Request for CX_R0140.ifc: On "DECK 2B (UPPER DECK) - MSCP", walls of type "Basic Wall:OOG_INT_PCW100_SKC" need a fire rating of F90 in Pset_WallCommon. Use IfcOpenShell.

First a look at what the model holds.

```python
import ifcopenshell
import ifcopenshell.util.element

model = ifcopenshell.open("CX_R0140.ifc")
print(model.schema)
storey = next(s for s in model.by_type("IfcBuildingStorey") if s.Name == "DECK 2B (UPPER DECK) - MSCP")
walls = [e for e in ifcopenshell.util.element.get_decomposition(storey) if e.is_a("IfcWall")]
seen = {}
for e in walls:
    element_type = ifcopenshell.util.element.get_type(e)
    key = (element_type.Name if element_type != e and element_type else None, ifcopenshell.util.element.get_pset(e, "Pset_WallCommon", "FireRating"))
    seen[key] = seen.get(key, 0) + 1
for (name, value), count in sorted(seen.items(), key=str):
    print(count, "x", name, "|", value)
```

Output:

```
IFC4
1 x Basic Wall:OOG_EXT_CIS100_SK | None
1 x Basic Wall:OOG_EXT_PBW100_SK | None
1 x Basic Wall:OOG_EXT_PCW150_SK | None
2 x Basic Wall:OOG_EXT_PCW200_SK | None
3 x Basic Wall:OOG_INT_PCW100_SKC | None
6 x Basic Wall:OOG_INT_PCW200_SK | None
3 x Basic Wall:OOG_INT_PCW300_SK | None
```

```python
import ifcopenshell
import ifcopenshell.api.pset
import ifcopenshell.util.element

model = ifcopenshell.open("CX_R0140.ifc")

storey = next(s for s in model.by_type("IfcBuildingStorey") if s.Name == "DECK 2B (UPPER DECK) - MSCP")
walls = [e for e in ifcopenshell.util.element.get_decomposition(storey) if e.is_a("IfcWall")]

count = 0
for e in walls:
    element_type = ifcopenshell.util.element.get_type(e)
    if element_type in (None, e) or element_type.Name != "Basic Wall:OOG_INT_PCW100_SKC":
        continue
    # add_pset returns the element's existing set when there is one.
    pset = ifcopenshell.api.pset.add_pset(model, product=e, name="Pset_WallCommon")
    ifcopenshell.api.pset.edit_pset(model, pset=pset, properties={"FireRating": "F90"})
    count += 1

print(count, "walls updated")

model.write("CX_R0140_edited.ifc")
```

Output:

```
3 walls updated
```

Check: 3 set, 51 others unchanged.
